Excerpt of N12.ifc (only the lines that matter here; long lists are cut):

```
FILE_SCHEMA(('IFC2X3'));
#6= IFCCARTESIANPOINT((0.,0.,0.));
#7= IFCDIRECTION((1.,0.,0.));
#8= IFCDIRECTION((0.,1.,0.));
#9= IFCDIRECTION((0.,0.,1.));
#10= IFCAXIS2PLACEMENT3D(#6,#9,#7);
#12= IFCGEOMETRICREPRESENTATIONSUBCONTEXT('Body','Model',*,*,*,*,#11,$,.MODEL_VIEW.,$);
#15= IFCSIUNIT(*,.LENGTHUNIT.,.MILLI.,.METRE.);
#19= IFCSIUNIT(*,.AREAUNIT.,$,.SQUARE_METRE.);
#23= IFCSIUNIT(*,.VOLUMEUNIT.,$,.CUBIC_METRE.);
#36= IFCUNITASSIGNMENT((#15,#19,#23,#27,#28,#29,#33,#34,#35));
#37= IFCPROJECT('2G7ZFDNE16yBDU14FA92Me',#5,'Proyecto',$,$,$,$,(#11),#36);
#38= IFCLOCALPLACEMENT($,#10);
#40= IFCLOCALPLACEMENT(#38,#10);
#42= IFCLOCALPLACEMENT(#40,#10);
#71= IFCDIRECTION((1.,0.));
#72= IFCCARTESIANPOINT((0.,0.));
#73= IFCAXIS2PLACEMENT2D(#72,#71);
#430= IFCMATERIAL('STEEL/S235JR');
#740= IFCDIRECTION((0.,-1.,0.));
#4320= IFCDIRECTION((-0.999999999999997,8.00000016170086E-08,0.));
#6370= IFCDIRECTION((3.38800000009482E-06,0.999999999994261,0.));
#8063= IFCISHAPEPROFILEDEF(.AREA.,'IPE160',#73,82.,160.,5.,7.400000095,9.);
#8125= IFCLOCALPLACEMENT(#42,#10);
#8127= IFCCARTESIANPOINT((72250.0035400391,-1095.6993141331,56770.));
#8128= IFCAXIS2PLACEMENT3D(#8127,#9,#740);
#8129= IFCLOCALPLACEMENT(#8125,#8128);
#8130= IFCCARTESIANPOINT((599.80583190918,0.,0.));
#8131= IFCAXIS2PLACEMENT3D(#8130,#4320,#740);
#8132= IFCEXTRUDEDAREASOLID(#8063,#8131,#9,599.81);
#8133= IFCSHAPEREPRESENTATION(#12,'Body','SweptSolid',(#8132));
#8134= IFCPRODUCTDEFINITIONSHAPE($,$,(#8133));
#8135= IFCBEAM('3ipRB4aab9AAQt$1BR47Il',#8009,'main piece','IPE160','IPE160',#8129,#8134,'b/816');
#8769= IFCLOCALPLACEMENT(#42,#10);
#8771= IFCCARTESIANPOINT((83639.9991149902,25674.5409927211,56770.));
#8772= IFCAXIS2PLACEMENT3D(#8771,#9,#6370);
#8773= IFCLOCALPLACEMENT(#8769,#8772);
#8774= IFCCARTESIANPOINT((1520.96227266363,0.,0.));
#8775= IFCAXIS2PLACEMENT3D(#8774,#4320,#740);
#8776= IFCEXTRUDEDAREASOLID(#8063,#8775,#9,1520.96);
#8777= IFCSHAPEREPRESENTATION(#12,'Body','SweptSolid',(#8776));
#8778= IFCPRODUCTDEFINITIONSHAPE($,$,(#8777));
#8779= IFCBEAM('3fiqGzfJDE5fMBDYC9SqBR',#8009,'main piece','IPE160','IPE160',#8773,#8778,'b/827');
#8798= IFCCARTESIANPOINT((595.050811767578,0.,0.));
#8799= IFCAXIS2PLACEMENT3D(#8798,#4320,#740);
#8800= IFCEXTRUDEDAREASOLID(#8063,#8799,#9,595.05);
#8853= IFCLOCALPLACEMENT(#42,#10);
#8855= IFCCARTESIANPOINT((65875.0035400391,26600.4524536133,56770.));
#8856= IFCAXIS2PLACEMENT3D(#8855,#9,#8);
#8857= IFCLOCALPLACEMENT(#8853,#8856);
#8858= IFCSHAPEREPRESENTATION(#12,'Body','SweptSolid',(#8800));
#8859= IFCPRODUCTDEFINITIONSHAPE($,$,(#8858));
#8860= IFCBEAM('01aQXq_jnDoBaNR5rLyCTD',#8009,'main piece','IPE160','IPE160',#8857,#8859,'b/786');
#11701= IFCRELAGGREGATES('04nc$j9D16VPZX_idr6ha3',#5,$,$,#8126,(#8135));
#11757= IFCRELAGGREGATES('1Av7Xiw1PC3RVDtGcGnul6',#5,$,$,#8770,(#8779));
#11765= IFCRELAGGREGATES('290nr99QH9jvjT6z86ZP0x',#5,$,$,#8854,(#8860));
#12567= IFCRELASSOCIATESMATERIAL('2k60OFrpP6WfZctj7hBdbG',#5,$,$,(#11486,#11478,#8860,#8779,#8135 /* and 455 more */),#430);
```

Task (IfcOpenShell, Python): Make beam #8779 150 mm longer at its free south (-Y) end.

```python
import ifcopenshell
import ifcopenshell.util.representation

model = ifcopenshell.open("N12.ifc")

member = model.by_id(8779)
change = 150.0

# The extrusion runs towards the end named, so only its depth changes.
body = ifcopenshell.util.representation.get_representation(member, "Model", "Body")
solid = body.Items[0]
old_length = solid.Depth
solid.Depth += change

print(f"length {old_length:g} -> {solid.Depth:g}")

model.write("N12_updated.ifc")
```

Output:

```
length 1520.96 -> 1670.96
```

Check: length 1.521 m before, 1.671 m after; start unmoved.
